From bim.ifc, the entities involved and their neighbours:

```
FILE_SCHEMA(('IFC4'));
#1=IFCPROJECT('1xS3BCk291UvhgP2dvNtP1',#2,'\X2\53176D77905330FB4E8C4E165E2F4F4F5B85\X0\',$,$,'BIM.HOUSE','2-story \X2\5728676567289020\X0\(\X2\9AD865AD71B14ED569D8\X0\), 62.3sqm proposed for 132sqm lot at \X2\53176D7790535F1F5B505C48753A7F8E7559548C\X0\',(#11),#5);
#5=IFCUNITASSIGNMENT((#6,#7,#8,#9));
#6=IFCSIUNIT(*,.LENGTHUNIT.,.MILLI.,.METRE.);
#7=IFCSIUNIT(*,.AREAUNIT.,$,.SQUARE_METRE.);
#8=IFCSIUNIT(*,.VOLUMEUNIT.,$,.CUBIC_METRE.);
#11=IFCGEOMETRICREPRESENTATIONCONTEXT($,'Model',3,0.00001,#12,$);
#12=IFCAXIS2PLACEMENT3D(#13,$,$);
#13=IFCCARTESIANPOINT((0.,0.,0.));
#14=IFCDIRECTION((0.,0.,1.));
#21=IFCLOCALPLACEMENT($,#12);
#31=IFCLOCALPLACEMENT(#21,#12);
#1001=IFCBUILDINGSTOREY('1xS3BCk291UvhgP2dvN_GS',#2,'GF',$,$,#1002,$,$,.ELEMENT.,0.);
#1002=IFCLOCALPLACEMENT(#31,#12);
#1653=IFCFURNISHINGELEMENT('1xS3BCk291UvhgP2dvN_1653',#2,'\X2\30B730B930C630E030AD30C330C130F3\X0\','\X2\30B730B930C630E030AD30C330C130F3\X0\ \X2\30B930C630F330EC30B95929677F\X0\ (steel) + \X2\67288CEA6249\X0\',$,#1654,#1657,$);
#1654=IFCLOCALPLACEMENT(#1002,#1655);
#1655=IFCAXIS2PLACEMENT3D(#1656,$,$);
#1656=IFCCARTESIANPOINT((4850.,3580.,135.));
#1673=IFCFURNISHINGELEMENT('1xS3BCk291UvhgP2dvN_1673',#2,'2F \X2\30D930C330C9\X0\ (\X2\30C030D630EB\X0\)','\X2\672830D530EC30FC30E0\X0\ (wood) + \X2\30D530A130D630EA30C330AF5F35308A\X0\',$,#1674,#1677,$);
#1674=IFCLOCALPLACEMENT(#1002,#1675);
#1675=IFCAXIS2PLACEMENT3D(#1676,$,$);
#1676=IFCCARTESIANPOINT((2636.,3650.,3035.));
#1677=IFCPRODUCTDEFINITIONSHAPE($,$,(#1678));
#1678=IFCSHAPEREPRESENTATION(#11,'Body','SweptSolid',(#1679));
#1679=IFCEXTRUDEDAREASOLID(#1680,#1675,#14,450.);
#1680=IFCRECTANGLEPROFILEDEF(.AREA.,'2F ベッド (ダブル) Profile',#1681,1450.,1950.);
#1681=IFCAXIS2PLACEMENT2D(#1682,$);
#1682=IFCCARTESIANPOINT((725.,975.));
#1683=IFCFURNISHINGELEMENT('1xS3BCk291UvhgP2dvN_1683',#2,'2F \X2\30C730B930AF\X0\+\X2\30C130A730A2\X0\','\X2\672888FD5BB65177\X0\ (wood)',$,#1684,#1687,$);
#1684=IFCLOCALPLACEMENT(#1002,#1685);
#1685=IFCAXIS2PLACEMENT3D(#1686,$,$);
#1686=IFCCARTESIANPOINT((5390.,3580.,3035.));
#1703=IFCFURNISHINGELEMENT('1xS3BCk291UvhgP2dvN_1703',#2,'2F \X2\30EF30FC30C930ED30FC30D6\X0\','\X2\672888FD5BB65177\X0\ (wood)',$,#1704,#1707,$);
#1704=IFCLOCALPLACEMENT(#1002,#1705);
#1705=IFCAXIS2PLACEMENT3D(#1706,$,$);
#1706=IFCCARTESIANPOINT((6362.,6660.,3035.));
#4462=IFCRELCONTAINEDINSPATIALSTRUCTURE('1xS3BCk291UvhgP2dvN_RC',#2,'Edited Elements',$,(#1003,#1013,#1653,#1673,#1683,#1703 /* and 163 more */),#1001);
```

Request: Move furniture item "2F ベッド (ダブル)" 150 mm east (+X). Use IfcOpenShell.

```python
import ifcopenshell
import ifcopenshell.api.geometry
import ifcopenshell.util.placement

model = ifcopenshell.open("bim.ifc")

item = model.by_guid("1xS3BCk291UvhgP2dvN_1673")
matrix = ifcopenshell.util.placement.get_local_placement(item.ObjectPlacement)
matrix[0, 3] += 150.0
ifcopenshell.api.geometry.edit_object_placement(model, product=item, matrix=matrix, is_si=False)

print(ifcopenshell.util.placement.get_local_placement(item.ObjectPlacement).round(3) + 0.0)

model.write("bim_v2.ifc")
```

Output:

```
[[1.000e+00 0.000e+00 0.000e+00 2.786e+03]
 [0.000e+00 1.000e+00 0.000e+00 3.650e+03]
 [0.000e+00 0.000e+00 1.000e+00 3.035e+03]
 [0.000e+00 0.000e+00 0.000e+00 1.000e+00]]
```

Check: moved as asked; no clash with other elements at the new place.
